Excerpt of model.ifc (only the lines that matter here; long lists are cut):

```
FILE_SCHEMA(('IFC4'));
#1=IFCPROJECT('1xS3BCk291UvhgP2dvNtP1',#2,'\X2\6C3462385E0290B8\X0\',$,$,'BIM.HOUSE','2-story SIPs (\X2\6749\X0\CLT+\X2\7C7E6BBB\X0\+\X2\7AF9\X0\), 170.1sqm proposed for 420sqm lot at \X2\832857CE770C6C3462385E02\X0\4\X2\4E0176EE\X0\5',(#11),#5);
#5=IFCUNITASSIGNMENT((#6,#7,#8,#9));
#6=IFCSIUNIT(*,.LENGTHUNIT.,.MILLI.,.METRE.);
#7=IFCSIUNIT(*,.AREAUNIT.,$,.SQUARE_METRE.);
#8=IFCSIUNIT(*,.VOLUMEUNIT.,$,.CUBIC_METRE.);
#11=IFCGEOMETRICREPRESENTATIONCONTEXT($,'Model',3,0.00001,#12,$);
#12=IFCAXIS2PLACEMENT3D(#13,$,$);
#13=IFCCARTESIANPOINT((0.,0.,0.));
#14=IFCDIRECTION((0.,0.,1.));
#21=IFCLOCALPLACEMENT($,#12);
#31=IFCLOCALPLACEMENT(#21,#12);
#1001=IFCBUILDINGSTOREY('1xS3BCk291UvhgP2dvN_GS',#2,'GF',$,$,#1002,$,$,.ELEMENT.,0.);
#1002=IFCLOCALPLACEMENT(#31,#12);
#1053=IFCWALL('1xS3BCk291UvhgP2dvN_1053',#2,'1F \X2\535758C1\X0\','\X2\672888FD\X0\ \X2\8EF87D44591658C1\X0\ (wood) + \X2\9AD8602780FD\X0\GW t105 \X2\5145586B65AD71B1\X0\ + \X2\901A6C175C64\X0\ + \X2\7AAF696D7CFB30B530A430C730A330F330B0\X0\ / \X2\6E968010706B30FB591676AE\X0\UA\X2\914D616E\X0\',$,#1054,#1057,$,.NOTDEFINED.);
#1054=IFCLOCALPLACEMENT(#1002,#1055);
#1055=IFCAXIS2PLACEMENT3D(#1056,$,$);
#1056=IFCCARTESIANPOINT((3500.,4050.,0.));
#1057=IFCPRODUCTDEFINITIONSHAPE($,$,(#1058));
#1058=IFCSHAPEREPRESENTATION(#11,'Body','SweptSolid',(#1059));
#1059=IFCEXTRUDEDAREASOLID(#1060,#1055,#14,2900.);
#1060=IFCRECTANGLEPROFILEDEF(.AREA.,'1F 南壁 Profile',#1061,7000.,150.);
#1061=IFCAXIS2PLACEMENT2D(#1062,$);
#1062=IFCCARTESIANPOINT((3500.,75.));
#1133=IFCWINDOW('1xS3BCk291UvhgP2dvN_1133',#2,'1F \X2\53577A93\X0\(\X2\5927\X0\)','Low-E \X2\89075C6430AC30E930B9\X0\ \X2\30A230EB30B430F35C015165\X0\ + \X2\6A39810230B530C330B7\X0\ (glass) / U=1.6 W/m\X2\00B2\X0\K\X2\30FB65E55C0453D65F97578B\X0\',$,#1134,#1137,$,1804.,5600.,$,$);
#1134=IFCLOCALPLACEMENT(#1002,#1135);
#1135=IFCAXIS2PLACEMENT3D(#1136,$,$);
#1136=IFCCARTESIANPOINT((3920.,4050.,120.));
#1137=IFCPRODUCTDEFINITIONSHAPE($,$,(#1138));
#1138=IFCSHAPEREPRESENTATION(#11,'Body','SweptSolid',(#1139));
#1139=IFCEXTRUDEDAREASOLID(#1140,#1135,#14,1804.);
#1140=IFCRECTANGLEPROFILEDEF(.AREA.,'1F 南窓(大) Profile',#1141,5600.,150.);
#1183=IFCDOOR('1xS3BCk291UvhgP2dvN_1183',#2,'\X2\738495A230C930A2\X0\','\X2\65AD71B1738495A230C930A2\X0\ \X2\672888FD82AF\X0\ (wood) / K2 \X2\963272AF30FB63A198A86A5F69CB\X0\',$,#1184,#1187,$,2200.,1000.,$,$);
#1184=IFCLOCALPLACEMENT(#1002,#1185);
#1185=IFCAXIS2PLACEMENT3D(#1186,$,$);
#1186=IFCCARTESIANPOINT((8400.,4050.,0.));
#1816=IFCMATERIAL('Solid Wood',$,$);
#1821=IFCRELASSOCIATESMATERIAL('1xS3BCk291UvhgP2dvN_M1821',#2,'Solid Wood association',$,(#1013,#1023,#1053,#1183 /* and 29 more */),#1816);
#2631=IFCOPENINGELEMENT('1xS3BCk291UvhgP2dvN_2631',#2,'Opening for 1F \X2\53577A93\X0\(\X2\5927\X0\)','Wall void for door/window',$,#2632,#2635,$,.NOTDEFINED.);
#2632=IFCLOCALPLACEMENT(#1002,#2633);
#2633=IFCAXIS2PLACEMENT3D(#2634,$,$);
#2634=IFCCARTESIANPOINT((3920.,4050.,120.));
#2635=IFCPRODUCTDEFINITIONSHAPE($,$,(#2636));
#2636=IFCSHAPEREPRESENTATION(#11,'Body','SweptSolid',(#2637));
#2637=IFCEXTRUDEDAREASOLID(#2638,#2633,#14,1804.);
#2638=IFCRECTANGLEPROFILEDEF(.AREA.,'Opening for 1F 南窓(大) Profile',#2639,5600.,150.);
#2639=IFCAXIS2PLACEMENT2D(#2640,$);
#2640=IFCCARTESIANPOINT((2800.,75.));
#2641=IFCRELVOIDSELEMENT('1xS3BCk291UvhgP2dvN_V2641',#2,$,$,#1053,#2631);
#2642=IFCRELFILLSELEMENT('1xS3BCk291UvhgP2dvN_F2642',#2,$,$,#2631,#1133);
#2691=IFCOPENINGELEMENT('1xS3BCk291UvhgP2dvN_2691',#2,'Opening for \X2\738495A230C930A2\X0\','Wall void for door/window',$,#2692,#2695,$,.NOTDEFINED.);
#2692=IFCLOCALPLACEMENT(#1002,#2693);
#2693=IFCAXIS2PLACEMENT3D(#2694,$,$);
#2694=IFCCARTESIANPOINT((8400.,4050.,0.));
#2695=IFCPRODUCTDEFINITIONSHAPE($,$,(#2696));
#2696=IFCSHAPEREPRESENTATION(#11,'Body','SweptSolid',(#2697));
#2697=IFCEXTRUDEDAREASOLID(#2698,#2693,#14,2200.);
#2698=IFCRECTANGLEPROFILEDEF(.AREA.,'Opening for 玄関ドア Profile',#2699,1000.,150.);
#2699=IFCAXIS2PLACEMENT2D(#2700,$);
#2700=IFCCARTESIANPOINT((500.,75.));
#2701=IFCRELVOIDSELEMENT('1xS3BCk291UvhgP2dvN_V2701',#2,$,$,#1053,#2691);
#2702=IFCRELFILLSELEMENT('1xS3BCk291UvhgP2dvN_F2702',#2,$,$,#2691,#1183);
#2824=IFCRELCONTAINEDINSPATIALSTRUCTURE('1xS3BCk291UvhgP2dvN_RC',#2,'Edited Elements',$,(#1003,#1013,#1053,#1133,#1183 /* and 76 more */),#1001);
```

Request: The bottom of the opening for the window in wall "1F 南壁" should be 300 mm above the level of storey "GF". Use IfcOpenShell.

```python
import numpy as np
import ifcopenshell
import ifcopenshell.api.geometry
import ifcopenshell.geom
import ifcopenshell.util.element
import ifcopenshell.util.placement
import ifcopenshell.util.shape
import ifcopenshell.util.unit

model = ifcopenshell.open("model.ifc")
unit_scale = ifcopenshell.util.unit.calculate_unit_scale(model)

window = model.by_guid("1xS3BCk291UvhgP2dvN_1133")
opening = window.FillsVoids[0].RelatingOpeningElement
storey = ifcopenshell.util.element.get_container(window, ifc_class="IfcBuildingStorey")
level = ifcopenshell.util.placement.get_local_placement(storey.ObjectPlacement)[2, 3]

# The opening's origin need not be at the sill, so measure its lowest point.
shape = ifcopenshell.geom.create_shape(ifcopenshell.geom.settings(), opening)
bottom = ifcopenshell.util.shape.get_shape_bottom_elevation(shape, shape.geometry) / unit_scale
dz = level + 300.0 - bottom

shift = np.array([0.0, 0.0, dz])
# The window is not placed relative to its opening, so move both.
for product in (opening, window):
    matrix = ifcopenshell.util.placement.get_local_placement(product.ObjectPlacement)
    matrix[:3, 3] += shift
    ifcopenshell.api.geometry.edit_object_placement(model, product=product, matrix=matrix, is_si=False)

print(f"moved by {dz * unit_scale:+.3f} m")

model.write("model_edited.ifc")
```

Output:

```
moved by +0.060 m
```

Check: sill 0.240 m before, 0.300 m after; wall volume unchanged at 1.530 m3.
